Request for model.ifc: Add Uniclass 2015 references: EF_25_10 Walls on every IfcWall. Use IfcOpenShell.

First a look at what the model holds.

```python
import ifcopenshell

model = ifcopenshell.open("model.ifc")
print(model.schema)
print("classifications:", [c.Name for c in model.by_type("IfcClassification")])
for ifc_class in ("IfcDoor", "IfcRoof", "IfcStair", "IfcWall", "IfcWindow"):
    print(ifc_class, len(model.by_type(ifc_class)))
```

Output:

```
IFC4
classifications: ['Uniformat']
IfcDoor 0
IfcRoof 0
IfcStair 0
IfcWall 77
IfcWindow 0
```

```python
import ifcopenshell
import ifcopenshell.api.classification

model = ifcopenshell.open("model.ifc")

system = ifcopenshell.api.classification.add_classification(model, classification="Uniclass 2015")

codes = {
    "IfcWall": ("EF_25_10", "Walls"),
}
for ifc_class, (code, name) in codes.items():
    products = model.by_type(ifc_class)
    ifcopenshell.api.classification.add_reference(
        model, products=products, classification=system, identification=code, name=name
    )
    print(code, len(products))

model.write("model_rev.ifc")
```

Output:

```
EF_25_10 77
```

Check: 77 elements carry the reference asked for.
